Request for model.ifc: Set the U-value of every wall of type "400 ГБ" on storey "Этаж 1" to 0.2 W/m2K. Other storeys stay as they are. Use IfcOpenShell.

First a look at what the model holds.

```python
import ifcopenshell
import ifcopenshell.util.element

model = ifcopenshell.open("model.ifc")
print(model.schema)
storey = next(s for s in model.by_type("IfcBuildingStorey") if s.Name == "Этаж 1")
walls = [e for e in ifcopenshell.util.element.get_decomposition(storey) if e.is_a("IfcWall")]
seen = {}
for e in walls:
    element_type = ifcopenshell.util.element.get_type(e)
    key = (element_type.Name if element_type != e and element_type else None, ifcopenshell.util.element.get_pset(e, "Pset_WallCommon", "ThermalTransmittance"))
    seen[key] = seen.get(key, 0) + 1
for (name, value), count in sorted(seen.items(), key=str):
    print(count, "x", name, "|", value)
```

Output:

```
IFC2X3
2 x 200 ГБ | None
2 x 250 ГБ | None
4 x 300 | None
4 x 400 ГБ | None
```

```python
import ifcopenshell
import ifcopenshell.api.pset
import ifcopenshell.util.element

model = ifcopenshell.open("model.ifc")

storey = next(s for s in model.by_type("IfcBuildingStorey") if s.Name == "Этаж 1")
walls = [e for e in ifcopenshell.util.element.get_decomposition(storey) if e.is_a("IfcWall")]

count = 0
for e in walls:
    element_type = ifcopenshell.util.element.get_type(e)
    if element_type in (None, e) or element_type.Name != "400 ГБ":
        continue
    # add_pset returns the element's existing set when there is one.
    pset = ifcopenshell.api.pset.add_pset(model, product=e, name="Pset_WallCommon")
    ifcopenshell.api.pset.edit_pset(model, pset=pset, properties={"ThermalTransmittance": 0.2})
    count += 1

print(count, "walls updated")

model.write("model_edited.ifc")
```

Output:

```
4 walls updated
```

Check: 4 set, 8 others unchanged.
